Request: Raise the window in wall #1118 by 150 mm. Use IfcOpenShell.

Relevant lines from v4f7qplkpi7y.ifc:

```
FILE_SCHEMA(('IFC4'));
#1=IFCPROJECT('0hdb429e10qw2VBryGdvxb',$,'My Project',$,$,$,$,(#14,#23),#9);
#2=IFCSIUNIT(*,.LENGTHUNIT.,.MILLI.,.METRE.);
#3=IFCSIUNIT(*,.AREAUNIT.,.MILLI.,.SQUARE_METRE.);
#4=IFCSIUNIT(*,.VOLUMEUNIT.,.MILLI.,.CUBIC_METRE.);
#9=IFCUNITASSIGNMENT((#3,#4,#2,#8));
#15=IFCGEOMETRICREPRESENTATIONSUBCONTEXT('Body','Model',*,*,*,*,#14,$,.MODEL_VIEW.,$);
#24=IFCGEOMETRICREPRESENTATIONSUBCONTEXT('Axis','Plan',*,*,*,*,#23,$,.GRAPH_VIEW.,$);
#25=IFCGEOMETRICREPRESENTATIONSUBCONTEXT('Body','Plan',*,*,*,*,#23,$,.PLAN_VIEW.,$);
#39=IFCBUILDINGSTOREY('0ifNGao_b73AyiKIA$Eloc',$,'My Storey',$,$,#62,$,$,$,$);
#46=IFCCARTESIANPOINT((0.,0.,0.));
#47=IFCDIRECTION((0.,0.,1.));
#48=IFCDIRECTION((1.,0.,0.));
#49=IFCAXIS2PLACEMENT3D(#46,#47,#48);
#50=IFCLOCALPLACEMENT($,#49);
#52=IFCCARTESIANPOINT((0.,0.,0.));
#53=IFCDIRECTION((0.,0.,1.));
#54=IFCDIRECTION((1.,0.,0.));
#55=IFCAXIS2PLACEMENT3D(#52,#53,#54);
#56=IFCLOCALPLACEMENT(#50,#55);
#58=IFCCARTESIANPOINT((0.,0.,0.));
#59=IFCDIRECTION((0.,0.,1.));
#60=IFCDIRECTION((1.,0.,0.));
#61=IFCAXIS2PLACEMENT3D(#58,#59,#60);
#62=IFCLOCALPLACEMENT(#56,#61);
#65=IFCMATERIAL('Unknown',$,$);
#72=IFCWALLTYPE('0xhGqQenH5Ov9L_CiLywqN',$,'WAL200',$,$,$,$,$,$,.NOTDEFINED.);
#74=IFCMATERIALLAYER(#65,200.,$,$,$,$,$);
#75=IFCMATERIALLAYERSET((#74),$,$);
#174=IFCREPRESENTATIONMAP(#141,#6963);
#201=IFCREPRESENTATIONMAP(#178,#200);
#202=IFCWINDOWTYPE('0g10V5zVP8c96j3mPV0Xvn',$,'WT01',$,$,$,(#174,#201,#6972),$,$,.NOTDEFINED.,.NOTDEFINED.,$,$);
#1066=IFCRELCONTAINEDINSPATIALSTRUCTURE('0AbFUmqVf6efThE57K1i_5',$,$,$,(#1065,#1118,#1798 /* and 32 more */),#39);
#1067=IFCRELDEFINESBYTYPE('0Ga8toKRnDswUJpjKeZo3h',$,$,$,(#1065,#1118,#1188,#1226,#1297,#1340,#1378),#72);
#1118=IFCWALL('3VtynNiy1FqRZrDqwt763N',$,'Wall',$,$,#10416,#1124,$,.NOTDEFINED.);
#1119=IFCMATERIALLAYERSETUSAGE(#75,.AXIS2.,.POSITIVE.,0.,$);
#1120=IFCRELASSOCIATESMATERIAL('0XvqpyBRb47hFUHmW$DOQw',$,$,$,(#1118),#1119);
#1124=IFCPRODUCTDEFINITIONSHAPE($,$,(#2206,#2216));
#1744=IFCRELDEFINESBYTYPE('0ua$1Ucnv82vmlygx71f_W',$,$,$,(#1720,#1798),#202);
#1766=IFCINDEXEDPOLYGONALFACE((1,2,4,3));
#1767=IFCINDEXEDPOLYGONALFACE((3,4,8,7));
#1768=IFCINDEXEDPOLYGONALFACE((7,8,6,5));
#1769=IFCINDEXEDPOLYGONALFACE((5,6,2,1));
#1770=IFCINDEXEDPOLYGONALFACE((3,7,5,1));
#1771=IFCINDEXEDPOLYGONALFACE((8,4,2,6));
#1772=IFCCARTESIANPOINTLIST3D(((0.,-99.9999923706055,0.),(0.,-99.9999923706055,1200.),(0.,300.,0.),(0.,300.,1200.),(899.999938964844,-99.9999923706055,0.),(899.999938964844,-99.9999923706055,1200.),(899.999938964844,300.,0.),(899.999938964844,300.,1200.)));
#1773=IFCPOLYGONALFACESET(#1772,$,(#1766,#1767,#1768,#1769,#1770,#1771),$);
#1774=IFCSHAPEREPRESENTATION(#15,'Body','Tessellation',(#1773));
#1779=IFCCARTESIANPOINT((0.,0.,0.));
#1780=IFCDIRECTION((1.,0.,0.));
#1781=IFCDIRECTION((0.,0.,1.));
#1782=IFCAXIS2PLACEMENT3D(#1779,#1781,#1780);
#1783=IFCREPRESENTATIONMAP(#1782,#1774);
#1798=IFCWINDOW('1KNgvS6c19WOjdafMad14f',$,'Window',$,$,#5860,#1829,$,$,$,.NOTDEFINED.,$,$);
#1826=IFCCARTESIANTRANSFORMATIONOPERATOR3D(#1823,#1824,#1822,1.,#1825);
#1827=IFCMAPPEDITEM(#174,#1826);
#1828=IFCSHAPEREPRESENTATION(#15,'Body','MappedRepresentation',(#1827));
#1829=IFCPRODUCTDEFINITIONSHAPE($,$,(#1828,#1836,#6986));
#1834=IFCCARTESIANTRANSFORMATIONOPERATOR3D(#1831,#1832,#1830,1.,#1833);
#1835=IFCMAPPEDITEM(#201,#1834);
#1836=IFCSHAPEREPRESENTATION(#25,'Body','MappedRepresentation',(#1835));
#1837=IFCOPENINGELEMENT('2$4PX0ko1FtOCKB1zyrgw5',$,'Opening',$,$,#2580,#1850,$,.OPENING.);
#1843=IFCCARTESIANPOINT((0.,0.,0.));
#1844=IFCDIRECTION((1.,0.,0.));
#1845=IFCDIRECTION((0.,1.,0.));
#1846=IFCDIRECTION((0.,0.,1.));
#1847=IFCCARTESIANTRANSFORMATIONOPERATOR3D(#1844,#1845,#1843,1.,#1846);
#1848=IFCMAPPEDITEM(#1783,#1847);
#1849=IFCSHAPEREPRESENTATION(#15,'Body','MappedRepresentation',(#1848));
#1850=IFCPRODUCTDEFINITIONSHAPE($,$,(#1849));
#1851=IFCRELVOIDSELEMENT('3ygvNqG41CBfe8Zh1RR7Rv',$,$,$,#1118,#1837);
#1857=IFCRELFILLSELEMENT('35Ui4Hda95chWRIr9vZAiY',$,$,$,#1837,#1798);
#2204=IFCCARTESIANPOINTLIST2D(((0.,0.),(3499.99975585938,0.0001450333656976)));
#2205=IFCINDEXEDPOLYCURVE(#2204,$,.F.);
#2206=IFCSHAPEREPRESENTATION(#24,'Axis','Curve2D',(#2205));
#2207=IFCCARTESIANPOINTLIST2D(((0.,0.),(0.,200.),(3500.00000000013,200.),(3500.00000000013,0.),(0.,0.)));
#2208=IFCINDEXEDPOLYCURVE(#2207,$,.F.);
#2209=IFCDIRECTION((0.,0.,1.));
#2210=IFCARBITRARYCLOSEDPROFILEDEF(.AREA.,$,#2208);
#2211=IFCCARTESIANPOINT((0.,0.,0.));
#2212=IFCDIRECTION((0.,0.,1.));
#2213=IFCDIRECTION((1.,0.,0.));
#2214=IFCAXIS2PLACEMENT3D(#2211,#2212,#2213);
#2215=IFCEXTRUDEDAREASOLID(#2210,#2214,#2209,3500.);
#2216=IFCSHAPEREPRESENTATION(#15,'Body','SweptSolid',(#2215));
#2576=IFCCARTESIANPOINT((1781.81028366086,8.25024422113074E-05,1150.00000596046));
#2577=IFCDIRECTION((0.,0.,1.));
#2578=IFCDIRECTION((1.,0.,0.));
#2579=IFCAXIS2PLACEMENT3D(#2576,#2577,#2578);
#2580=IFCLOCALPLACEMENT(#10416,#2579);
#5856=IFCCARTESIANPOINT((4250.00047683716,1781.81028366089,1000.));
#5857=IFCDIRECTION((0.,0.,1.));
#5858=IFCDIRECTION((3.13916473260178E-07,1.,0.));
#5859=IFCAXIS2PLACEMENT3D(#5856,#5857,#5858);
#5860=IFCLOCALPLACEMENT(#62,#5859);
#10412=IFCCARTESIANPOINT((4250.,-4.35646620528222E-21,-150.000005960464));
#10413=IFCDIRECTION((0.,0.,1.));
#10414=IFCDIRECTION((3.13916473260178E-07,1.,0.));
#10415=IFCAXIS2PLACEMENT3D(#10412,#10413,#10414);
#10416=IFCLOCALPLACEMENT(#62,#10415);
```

```python
import numpy as np
import ifcopenshell
import ifcopenshell.api.geometry
import ifcopenshell.util.placement
import ifcopenshell.util.unit

model = ifcopenshell.open("v4f7qplkpi7y.ifc")
unit_scale = ifcopenshell.util.unit.calculate_unit_scale(model)

window = model.by_guid("1KNgvS6c19WOjdafMad14f")
opening = window.FillsVoids[0].RelatingOpeningElement
dz = 0.15 / unit_scale

shift = np.array([0.0, 0.0, dz])
# The window is not placed relative to its opening, so move both.
for product in (opening, window):
    matrix = ifcopenshell.util.placement.get_local_placement(product.ObjectPlacement)
    matrix[:3, 3] += shift
    ifcopenshell.api.geometry.edit_object_placement(model, product=product, matrix=matrix, is_si=False)

print(f"moved by {dz * unit_scale:+.3f} m")

model.write("v4f7qplkpi7y_edited.ifc")
```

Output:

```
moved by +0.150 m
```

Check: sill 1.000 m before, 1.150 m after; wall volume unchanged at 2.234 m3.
